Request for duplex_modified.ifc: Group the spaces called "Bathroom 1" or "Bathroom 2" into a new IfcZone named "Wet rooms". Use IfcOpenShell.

First a look at what the model holds.

```python
import ifcopenshell

model = ifcopenshell.open("duplex_modified.ifc")
print(model.schema)
seen = {}
for space in model.by_type("IfcSpace"):
    seen[space.LongName] = seen.get(space.LongName, 0) + 1
for name, count in sorted(seen.items(), key=str):
    print(count, "x", name)
print("zones:", [z.Name for z in model.by_type("IfcZone")][:20])
```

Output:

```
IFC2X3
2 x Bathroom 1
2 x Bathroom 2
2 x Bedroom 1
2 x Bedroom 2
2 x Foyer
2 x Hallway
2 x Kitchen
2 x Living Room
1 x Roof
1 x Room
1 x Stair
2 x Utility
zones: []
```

```python
import ifcopenshell
import ifcopenshell.api.group
import ifcopenshell.api.root

model = ifcopenshell.open("duplex_modified.ifc")

names = {"Bathroom 1", "Bathroom 2"}
spaces = [s for s in model.by_type("IfcSpace") if s.LongName in names]

zone = ifcopenshell.api.root.create_entity(model, ifc_class="IfcZone", name="Wet rooms")
ifcopenshell.api.group.assign_group(model, products=spaces, group=zone)
print(len(spaces), "spaces in", zone.Name)

model.write("duplex_modified_updated.ifc")
```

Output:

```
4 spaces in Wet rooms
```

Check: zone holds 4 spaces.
